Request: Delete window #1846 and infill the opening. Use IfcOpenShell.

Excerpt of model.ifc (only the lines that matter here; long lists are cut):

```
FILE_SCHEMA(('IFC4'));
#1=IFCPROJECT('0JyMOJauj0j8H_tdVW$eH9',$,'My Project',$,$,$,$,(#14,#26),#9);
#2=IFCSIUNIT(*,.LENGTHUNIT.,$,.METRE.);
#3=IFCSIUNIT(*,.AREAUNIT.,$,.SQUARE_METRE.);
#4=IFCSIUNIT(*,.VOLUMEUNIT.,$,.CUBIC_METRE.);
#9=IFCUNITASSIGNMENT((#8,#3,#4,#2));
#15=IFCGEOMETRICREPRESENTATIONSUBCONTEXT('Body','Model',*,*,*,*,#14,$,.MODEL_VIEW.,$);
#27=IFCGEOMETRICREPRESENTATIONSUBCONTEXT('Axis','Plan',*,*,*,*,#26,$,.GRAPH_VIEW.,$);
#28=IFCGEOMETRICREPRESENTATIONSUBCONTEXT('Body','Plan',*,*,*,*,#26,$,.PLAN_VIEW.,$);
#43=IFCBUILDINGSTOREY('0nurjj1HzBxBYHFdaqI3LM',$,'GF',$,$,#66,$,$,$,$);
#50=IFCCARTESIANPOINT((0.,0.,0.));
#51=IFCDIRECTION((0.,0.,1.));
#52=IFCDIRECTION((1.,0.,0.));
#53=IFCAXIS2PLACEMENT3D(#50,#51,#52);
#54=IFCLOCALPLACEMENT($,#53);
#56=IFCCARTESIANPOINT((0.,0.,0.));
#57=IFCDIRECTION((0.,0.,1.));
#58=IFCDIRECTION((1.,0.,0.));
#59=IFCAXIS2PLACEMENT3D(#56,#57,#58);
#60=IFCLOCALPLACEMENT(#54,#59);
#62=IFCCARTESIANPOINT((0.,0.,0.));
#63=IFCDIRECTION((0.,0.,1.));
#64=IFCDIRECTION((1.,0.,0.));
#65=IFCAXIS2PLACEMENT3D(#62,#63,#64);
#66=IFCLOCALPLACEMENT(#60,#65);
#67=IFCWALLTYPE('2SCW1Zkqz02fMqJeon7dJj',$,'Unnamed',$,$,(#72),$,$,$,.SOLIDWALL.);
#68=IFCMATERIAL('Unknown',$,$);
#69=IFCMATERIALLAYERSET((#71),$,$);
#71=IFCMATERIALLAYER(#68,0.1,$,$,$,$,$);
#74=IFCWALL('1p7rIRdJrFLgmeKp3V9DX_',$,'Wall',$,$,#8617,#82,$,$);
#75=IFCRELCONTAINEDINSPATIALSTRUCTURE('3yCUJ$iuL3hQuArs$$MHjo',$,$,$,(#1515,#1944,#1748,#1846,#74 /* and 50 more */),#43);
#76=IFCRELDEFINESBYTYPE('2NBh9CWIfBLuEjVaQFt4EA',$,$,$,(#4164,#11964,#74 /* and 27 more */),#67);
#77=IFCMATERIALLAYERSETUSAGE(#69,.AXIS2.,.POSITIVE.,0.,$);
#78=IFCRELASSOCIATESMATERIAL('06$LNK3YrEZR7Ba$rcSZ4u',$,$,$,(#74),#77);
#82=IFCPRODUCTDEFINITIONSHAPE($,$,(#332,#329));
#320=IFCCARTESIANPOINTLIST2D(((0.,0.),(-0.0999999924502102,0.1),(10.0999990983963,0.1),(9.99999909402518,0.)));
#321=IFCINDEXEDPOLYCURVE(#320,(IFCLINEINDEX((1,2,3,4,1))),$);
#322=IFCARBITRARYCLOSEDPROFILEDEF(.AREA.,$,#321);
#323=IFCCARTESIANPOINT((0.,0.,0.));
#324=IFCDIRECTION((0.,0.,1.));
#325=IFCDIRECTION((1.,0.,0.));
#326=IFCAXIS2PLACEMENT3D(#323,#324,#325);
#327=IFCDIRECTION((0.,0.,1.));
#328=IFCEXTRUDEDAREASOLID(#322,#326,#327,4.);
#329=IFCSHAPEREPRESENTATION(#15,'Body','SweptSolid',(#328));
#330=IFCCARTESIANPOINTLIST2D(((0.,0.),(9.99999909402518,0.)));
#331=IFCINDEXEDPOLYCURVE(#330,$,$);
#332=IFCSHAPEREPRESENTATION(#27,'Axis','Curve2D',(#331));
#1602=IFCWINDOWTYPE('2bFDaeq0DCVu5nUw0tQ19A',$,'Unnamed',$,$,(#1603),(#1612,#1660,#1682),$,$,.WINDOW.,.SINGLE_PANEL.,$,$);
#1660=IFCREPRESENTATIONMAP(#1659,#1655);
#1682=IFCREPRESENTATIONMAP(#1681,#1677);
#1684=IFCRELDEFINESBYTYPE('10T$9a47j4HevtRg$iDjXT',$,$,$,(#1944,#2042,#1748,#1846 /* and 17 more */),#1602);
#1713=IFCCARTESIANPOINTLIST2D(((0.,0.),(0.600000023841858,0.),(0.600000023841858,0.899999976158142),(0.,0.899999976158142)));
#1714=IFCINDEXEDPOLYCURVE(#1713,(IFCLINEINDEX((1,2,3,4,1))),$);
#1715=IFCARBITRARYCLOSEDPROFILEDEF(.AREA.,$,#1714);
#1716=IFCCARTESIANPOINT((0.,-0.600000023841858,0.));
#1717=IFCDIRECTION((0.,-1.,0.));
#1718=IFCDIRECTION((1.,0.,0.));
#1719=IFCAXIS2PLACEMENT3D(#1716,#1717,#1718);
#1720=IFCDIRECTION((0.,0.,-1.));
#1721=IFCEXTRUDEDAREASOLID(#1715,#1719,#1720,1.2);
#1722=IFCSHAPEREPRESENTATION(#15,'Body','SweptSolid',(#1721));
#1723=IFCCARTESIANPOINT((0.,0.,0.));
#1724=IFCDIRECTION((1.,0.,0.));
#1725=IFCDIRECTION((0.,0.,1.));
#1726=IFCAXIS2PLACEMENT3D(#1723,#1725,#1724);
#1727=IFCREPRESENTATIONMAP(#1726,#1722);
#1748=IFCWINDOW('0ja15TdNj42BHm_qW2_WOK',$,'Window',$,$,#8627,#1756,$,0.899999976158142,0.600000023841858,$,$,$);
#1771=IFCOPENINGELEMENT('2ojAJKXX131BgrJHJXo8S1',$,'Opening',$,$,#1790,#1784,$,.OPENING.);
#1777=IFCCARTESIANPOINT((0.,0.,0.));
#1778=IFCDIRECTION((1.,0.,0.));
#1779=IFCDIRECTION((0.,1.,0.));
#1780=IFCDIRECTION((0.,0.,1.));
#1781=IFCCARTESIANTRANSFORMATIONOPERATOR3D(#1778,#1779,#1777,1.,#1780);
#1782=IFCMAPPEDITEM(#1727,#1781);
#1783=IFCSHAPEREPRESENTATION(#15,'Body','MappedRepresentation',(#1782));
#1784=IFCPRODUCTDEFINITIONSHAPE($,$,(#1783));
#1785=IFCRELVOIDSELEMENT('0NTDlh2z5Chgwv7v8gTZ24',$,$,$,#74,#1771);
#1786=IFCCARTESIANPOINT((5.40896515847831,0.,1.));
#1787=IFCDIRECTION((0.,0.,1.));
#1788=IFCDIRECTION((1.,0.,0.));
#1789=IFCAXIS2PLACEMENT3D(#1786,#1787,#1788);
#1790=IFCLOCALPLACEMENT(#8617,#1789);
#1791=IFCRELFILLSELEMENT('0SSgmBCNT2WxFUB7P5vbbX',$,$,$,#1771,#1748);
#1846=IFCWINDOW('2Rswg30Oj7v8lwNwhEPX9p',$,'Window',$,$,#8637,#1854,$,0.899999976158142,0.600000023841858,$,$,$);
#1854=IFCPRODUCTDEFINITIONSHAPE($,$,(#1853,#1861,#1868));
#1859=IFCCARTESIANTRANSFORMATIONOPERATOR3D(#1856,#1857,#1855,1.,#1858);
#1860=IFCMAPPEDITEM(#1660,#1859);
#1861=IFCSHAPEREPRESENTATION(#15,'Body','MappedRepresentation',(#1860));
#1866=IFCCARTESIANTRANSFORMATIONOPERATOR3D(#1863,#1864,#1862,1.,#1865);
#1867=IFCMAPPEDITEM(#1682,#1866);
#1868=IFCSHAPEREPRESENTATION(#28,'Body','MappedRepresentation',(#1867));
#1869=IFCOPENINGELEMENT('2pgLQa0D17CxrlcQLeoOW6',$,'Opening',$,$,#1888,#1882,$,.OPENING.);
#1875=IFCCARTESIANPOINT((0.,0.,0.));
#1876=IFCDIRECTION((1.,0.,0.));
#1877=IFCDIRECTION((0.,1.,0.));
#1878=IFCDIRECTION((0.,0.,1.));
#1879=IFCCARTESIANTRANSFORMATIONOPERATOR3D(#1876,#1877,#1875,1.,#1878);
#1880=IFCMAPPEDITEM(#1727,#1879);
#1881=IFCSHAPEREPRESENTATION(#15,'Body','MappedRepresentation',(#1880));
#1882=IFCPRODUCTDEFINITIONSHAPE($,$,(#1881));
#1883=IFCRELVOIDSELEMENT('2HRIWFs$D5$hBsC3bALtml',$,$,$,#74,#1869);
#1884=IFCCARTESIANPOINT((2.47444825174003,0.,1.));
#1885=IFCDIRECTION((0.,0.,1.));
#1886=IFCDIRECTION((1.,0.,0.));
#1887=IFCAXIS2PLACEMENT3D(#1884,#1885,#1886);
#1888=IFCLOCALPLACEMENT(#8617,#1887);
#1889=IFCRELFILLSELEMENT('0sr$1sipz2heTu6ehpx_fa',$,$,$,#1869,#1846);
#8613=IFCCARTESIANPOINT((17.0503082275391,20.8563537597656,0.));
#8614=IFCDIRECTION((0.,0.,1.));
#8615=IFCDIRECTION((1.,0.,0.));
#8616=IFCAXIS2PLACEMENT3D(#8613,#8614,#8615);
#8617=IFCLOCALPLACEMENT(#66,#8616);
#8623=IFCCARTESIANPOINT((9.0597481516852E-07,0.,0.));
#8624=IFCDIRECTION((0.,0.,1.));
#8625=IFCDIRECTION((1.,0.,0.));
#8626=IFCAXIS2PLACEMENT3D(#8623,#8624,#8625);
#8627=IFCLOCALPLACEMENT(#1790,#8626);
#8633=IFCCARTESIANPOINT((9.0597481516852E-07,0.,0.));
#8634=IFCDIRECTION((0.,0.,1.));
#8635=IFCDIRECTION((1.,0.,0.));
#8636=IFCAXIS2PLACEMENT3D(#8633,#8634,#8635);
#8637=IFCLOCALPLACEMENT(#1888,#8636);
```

```python
import ifcopenshell
import ifcopenshell.api.feature
import ifcopenshell.api.root
import ifcopenshell.geom
import ifcopenshell.util.shape

model = ifcopenshell.open("model.ifc")
settings = ifcopenshell.geom.settings()


def volume(element):
    """Net volume in cubic metres, openings subtracted."""
    shape = ifcopenshell.geom.create_shape(settings, element)
    return ifcopenshell.util.shape.get_volume(shape.geometry)


window = model.by_id(1846)
opening = window.FillsVoids[0].RelatingOpeningElement
wall = opening.VoidsElements[0].RelatingBuildingElement
before = volume(wall)

ifcopenshell.api.root.remove_product(model, product=window)
ifcopenshell.api.feature.remove_feature(model, feature=opening)

after = volume(wall)

print(f"wall volume {before:.3f} -> {after:.3f} m3")

model.write("model-out.ifc")
```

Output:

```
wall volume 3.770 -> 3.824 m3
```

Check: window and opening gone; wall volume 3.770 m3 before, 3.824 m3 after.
